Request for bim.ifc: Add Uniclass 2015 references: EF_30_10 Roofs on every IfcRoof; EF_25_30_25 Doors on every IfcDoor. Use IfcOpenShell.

First a look at what the model holds.

```python
import ifcopenshell

model = ifcopenshell.open("bim.ifc")
print(model.schema)
print("classifications:", [c.Name for c in model.by_type("IfcClassification")])
for ifc_class in ("IfcDoor", "IfcRoof", "IfcStair", "IfcWall", "IfcWindow"):
    print(ifc_class, len(model.by_type(ifc_class)))
```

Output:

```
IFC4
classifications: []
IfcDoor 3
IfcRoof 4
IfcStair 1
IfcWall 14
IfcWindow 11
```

```python
import ifcopenshell
import ifcopenshell.api.classification

model = ifcopenshell.open("bim.ifc")

system = ifcopenshell.api.classification.add_classification(model, classification="Uniclass 2015")

codes = {
    "IfcRoof": ("EF_30_10", "Roofs"),
    "IfcDoor": ("EF_25_30_25", "Doors"),
}
for ifc_class, (code, name) in codes.items():
    products = model.by_type(ifc_class)
    ifcopenshell.api.classification.add_reference(
        model, products=products, classification=system, identification=code, name=name
    )
    print(code, len(products))

model.write("bim-out.ifc")
```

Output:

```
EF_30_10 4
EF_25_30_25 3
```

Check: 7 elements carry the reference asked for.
